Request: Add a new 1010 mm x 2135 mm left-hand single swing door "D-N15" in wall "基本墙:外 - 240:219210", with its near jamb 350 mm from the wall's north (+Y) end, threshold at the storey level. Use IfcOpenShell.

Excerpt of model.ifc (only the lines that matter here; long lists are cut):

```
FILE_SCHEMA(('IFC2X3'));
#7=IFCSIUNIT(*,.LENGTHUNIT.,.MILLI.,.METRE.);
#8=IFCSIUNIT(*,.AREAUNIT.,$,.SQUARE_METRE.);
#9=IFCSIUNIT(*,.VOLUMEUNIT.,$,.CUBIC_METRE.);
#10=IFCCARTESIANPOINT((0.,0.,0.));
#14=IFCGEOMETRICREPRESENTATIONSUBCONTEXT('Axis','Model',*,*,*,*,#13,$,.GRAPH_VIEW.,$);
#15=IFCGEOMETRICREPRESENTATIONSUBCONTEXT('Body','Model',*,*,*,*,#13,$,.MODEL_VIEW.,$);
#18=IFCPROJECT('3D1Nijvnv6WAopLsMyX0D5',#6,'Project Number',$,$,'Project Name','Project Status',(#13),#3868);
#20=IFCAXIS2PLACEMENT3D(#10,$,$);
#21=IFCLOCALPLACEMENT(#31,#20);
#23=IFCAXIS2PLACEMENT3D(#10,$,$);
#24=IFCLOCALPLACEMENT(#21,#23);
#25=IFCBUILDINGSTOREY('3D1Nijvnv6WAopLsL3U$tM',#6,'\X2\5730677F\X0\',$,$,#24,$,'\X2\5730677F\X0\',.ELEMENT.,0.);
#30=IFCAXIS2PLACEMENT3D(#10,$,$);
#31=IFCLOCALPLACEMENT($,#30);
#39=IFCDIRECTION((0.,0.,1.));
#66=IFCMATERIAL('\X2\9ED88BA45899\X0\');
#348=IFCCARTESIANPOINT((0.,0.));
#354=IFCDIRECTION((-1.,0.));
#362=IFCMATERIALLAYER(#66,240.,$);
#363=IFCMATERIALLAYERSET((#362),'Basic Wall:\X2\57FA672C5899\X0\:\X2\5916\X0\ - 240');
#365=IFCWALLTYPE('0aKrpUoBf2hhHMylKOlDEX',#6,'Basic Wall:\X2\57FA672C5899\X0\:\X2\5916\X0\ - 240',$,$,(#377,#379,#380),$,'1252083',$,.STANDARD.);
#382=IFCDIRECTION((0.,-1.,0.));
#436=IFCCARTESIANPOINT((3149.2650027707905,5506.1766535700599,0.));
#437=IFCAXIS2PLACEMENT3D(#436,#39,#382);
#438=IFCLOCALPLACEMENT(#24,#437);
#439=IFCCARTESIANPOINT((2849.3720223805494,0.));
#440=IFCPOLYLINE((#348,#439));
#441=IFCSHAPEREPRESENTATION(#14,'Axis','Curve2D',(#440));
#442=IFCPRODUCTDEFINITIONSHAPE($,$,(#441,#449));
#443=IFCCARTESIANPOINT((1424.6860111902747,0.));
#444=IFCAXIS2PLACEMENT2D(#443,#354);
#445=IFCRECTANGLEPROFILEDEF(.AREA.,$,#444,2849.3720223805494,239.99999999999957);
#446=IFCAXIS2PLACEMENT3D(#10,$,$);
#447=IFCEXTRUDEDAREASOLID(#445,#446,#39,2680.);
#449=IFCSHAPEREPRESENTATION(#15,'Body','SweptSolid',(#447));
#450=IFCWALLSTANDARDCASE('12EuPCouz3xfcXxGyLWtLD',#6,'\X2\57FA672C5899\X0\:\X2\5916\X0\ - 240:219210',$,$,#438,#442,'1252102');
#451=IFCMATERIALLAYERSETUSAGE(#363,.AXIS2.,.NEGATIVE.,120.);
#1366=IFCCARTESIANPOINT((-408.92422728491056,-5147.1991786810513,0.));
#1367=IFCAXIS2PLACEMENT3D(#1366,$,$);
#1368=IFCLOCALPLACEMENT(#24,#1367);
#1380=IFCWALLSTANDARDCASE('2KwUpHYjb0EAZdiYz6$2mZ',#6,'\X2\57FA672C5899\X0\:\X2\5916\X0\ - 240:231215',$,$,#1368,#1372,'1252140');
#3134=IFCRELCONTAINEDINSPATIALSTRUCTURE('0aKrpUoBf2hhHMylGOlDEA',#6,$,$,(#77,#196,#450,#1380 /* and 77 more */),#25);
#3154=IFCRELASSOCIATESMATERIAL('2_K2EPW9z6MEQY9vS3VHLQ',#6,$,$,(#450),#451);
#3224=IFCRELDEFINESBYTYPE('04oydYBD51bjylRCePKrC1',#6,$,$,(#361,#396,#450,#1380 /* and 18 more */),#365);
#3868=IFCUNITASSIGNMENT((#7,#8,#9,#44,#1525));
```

```python
import numpy as np
import ifcopenshell
import ifcopenshell.api.feature
import ifcopenshell.api.geometry
import ifcopenshell.api.root
import ifcopenshell.api.spatial
import ifcopenshell.api.type
import ifcopenshell.geom
import ifcopenshell.util.element
import ifcopenshell.util.placement
import ifcopenshell.util.representation
import ifcopenshell.util.shape
import ifcopenshell.util.unit

model = ifcopenshell.open("model.ifc")
unit_scale = ifcopenshell.util.unit.calculate_unit_scale(model)
settings = ifcopenshell.geom.settings()


def volume(element):
    """Net volume in cubic metres, openings subtracted."""
    shape = ifcopenshell.geom.create_shape(settings, element)
    return ifcopenshell.util.shape.get_volume(shape.geometry)


wall = model.by_id(450)
storey = ifcopenshell.util.element.get_container(wall, ifc_class="IfcBuildingStorey")
context = ifcopenshell.util.representation.get_context(model, "Model", "Body", "MODEL_VIEW")
before = volume(wall)

width, height, from_end, sill = 1.01, 2.135, 0.35, 0.0  # metres

# The wall runs along its own X axis, and the end named is its -X end.
wall_shape = ifcopenshell.geom.create_shape(settings, wall)
x, y, z = ifcopenshell.util.shape.get_vertices(wall_shape.geometry).T
start = x.min() + from_end
face, thickness = float(y.min()), float(y.max() - y.min())
wall_matrix = ifcopenshell.util.placement.get_local_placement(wall.ObjectPlacement)
level = ifcopenshell.util.placement.get_local_placement(storey.ObjectPlacement)[2, 3]


def in_wall(x, y):
    """Placement at x, y metres in the wall's axes, at sill height."""
    matrix = wall_matrix.copy()
    matrix[:, 3] = wall_matrix @ np.array([x / unit_scale, y / unit_scale, 0.0, 1.0])
    matrix[2, 3] = level + sill / unit_scale
    return matrix


# Opening: a box that overshoots both wall faces by 50 mm.
opening = ifcopenshell.api.root.create_entity(model, ifc_class="IfcOpeningElement")
box = ifcopenshell.api.geometry.add_wall_representation(
    model, context=context, length=width, height=height, thickness=thickness + 0.1
)
ifcopenshell.api.geometry.assign_representation(model, product=opening, representation=box)
ifcopenshell.api.geometry.edit_object_placement(model, product=opening, matrix=in_wall(start, face - 0.05), is_si=False)
ifcopenshell.api.feature.add_feature(model, feature=opening, element=wall)

door = ifcopenshell.api.root.create_entity(model, ifc_class="IfcDoor", name="D-N15")
door.OverallWidth, door.OverallHeight = width / unit_scale, height / unit_scale
body = ifcopenshell.api.geometry.add_door_representation(
    model,
    context=context,
    overall_width=door.OverallWidth,
    overall_height=door.OverallHeight,
    operation_type="SINGLE_SWING_LEFT",
    lining_properties={"LiningDepth": thickness / unit_scale, "ThresholdDepth": thickness / unit_scale},
)
ifcopenshell.api.geometry.assign_representation(model, product=door, representation=body)
ifcopenshell.api.spatial.assign_container(model, products=[door], relating_structure=storey)
fills = ifcopenshell.api.feature.add_filling(model, opening=opening, element=door)
fills.OwnerHistory = door.OwnerHistory  # required in IFC2X3

# IFC2X3 keeps the operation on the door style.
style = ifcopenshell.api.root.create_entity(model, ifc_class="IfcDoorStyle", name="D-N15")
style.OperationType, style.ConstructionType = "SINGLE_SWING_LEFT", "NOTDEFINED"
style.ParameterTakesPrecedence = style.Sizeable = False
ifcopenshell.api.type.assign_type(model, related_objects=[door], relating_type=style)

# The lining spans the wall, so the door starts at the wall face.
ifcopenshell.api.geometry.edit_object_placement(model, product=door, matrix=in_wall(start, face), is_si=False)

after = volume(wall)

print(f"wall volume {before:.3f} -> {after:.3f} m3")

model.write("model-out.ifc")
```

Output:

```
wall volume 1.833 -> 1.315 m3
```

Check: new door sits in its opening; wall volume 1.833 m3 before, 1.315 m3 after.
